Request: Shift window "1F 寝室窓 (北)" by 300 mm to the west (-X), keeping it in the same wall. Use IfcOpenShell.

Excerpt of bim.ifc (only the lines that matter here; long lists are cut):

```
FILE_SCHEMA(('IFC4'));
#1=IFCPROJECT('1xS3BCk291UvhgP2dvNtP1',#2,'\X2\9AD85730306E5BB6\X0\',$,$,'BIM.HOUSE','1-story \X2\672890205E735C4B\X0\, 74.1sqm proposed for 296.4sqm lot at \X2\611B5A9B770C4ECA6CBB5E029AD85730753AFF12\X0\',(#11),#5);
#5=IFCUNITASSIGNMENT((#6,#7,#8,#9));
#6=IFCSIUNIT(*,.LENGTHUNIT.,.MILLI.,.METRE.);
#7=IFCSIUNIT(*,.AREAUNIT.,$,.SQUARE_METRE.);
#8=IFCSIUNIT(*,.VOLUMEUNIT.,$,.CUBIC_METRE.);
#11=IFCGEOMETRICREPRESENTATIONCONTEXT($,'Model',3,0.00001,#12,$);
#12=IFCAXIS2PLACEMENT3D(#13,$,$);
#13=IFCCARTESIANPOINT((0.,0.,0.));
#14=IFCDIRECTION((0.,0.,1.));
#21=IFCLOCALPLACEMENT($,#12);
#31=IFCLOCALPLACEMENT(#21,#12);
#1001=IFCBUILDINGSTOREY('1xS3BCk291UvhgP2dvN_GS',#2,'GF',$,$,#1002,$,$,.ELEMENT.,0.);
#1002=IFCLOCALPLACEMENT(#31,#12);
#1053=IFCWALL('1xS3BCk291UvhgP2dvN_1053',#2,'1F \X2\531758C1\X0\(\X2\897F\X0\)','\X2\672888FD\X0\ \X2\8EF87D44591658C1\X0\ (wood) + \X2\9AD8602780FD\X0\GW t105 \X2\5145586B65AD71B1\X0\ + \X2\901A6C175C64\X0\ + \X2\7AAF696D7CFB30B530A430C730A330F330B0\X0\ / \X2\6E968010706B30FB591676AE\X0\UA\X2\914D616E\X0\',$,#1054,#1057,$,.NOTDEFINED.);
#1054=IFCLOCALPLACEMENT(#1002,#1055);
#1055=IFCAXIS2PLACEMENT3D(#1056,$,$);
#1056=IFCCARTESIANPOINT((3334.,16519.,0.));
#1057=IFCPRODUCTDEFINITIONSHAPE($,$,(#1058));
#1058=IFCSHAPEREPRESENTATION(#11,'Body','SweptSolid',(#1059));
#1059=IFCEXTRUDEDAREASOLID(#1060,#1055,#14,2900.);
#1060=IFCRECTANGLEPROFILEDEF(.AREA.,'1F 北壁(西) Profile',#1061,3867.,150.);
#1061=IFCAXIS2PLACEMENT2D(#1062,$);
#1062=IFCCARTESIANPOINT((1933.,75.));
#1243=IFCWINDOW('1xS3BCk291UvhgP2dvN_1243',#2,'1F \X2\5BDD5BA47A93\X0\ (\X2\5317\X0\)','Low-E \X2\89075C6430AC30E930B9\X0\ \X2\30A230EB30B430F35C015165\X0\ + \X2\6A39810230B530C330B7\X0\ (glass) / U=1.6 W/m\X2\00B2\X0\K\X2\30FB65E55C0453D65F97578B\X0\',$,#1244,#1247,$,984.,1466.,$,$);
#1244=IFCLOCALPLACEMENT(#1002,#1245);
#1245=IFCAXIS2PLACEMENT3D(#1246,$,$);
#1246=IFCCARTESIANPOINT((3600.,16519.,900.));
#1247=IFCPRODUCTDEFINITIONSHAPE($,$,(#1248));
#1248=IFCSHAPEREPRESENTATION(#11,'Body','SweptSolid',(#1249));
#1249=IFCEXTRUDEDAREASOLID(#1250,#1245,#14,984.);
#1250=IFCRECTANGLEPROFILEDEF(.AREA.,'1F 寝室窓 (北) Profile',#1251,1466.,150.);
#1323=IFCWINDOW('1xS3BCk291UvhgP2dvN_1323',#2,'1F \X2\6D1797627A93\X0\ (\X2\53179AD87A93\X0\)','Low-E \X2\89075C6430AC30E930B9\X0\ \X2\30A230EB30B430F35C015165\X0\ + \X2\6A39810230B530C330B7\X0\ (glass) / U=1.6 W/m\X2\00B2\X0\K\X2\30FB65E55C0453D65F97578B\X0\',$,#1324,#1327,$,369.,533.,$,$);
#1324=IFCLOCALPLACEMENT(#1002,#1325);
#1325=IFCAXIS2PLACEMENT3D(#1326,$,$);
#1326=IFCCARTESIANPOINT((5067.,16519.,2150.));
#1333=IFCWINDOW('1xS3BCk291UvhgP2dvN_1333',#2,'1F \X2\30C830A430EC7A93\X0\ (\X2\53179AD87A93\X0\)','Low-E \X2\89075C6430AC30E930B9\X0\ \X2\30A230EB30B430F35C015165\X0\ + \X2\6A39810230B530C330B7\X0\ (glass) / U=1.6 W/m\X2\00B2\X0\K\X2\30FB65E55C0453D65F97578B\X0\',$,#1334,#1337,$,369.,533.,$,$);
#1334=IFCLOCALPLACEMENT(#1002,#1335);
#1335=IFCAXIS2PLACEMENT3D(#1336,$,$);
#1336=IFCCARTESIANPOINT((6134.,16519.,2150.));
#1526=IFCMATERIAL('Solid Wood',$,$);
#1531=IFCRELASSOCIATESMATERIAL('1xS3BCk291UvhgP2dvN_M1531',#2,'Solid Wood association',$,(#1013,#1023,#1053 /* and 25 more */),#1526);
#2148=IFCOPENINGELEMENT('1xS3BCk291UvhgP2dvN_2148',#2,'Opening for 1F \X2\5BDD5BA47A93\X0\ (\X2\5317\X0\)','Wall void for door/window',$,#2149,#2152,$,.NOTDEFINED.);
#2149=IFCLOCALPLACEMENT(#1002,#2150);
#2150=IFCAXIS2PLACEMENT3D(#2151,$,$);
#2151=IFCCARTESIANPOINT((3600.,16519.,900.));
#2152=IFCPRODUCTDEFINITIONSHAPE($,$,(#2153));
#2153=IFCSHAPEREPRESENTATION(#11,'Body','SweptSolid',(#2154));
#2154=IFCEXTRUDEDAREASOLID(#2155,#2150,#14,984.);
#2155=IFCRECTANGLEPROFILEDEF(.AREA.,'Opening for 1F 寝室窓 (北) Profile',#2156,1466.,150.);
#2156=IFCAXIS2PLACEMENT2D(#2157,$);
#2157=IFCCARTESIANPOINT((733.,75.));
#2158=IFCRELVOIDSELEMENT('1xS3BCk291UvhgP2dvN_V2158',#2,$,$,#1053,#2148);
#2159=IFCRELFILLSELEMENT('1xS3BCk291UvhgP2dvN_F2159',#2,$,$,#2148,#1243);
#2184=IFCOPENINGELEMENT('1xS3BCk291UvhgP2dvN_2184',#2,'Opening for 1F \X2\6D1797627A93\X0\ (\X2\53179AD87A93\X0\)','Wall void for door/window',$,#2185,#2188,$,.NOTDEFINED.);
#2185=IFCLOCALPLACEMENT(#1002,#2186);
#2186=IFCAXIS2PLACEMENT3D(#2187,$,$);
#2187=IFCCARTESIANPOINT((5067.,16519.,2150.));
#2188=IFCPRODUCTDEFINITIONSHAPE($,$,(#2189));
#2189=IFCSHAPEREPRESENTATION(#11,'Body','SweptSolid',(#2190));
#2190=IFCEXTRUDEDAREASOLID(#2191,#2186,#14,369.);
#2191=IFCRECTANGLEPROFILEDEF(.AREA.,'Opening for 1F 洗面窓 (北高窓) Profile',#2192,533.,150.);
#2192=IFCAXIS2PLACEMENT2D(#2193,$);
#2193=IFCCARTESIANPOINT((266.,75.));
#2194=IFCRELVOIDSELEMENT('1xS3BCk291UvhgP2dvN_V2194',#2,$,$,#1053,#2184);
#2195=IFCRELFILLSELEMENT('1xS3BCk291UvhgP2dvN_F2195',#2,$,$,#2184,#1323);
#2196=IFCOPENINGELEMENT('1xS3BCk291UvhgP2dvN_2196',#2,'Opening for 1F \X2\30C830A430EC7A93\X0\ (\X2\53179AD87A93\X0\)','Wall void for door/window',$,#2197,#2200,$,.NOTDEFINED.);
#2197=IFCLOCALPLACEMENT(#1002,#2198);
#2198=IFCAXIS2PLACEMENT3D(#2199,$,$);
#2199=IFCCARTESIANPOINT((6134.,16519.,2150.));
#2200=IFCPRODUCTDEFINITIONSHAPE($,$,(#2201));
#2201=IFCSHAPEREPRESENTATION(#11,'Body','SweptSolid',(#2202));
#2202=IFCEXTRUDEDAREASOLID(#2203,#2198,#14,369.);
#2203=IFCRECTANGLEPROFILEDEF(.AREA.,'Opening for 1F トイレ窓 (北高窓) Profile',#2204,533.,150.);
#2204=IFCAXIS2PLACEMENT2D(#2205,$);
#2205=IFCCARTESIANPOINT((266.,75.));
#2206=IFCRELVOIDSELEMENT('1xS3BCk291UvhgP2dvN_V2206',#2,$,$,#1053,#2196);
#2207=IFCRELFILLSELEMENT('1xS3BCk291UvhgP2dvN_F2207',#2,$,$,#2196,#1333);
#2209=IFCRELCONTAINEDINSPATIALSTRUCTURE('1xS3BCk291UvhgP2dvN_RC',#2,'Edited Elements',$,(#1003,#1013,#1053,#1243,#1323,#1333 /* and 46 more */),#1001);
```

```python
import ifcopenshell
import ifcopenshell.api.geometry
import ifcopenshell.util.placement

model = ifcopenshell.open("bim.ifc")

window = model.by_guid("1xS3BCk291UvhgP2dvN_1243")
opening = window.FillsVoids[0].RelatingOpeningElement
wall = opening.VoidsElements[0].RelatingBuildingElement

wall_matrix = ifcopenshell.util.placement.get_local_placement(wall.ObjectPlacement)
shift = wall_matrix[:3, 0] * -300.0
before = ifcopenshell.util.placement.get_local_placement(window.ObjectPlacement)[:3, 3].copy()

# The window is not placed relative to its opening, so move both.
for product in (opening, window):
    matrix = ifcopenshell.util.placement.get_local_placement(product.ObjectPlacement)
    matrix[:3, 3] += shift
    ifcopenshell.api.geometry.edit_object_placement(model, product=product, matrix=matrix, is_si=False)

after = ifcopenshell.util.placement.get_local_placement(window.ObjectPlacement)[:3, 3]
print("window moved by", (after - before).round(3) + 0.0)

model.write("bim_edited.ifc")
```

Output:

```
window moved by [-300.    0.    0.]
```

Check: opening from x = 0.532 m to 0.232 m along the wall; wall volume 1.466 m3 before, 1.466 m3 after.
